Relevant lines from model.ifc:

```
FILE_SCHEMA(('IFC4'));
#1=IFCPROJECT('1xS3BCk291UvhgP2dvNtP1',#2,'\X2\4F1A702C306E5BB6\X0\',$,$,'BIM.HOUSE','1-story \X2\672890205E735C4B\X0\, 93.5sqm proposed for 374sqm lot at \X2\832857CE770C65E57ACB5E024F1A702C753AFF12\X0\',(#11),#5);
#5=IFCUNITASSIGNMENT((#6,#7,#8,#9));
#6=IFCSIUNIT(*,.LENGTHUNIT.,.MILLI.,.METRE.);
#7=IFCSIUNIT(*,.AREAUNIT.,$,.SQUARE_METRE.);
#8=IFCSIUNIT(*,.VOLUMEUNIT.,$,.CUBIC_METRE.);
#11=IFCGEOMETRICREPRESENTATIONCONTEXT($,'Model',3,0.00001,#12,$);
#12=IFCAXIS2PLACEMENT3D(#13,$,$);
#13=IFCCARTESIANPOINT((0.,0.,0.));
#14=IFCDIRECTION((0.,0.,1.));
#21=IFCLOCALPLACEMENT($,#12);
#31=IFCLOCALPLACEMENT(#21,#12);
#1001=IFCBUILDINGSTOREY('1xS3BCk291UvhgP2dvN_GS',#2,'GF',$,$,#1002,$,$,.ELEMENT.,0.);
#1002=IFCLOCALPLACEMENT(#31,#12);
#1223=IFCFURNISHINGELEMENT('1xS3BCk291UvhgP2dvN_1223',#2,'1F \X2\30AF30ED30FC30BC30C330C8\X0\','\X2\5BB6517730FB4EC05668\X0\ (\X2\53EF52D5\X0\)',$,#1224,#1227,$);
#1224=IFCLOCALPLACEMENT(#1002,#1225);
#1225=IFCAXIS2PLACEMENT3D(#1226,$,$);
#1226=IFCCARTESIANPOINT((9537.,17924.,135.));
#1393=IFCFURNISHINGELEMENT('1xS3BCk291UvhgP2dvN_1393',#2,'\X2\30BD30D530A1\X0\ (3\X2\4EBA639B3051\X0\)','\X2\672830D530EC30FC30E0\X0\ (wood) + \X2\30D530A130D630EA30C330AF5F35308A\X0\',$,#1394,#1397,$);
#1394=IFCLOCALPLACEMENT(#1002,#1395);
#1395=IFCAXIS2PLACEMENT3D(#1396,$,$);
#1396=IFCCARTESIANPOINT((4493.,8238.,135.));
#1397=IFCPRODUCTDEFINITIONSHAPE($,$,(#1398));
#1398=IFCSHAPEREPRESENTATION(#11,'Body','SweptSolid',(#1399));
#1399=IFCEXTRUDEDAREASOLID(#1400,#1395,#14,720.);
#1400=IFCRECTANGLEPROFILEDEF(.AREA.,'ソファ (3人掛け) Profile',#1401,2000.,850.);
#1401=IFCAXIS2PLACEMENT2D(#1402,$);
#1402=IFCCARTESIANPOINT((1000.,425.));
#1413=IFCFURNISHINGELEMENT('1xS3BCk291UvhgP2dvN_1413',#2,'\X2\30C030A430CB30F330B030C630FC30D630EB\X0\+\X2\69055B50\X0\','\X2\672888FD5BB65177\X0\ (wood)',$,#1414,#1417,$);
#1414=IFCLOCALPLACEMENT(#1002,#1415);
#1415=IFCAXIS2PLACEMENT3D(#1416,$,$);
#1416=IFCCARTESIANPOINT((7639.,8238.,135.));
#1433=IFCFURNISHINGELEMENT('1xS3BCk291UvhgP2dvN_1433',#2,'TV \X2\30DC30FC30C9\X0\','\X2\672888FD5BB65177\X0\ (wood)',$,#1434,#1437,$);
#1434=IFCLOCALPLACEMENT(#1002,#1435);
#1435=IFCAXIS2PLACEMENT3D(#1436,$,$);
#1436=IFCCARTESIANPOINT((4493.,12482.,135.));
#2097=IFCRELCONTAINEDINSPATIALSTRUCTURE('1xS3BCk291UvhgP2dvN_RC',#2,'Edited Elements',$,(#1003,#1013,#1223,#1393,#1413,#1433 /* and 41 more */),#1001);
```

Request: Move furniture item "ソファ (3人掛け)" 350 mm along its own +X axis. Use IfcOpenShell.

```python
import ifcopenshell
import ifcopenshell.api.geometry
import ifcopenshell.util.placement

model = ifcopenshell.open("model.ifc")

item = model.by_guid("1xS3BCk291UvhgP2dvN_1393")
matrix = ifcopenshell.util.placement.get_local_placement(item.ObjectPlacement)
matrix[:3, 3] += matrix[:3, 0] * 350.0
ifcopenshell.api.geometry.edit_object_placement(model, product=item, matrix=matrix, is_si=False)

print(ifcopenshell.util.placement.get_local_placement(item.ObjectPlacement).round(3) + 0.0)

model.write("model_rev.ifc")
```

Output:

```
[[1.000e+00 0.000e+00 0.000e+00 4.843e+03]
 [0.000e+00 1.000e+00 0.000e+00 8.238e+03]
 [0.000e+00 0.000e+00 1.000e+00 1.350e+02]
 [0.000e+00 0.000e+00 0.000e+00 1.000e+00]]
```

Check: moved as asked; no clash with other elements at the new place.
